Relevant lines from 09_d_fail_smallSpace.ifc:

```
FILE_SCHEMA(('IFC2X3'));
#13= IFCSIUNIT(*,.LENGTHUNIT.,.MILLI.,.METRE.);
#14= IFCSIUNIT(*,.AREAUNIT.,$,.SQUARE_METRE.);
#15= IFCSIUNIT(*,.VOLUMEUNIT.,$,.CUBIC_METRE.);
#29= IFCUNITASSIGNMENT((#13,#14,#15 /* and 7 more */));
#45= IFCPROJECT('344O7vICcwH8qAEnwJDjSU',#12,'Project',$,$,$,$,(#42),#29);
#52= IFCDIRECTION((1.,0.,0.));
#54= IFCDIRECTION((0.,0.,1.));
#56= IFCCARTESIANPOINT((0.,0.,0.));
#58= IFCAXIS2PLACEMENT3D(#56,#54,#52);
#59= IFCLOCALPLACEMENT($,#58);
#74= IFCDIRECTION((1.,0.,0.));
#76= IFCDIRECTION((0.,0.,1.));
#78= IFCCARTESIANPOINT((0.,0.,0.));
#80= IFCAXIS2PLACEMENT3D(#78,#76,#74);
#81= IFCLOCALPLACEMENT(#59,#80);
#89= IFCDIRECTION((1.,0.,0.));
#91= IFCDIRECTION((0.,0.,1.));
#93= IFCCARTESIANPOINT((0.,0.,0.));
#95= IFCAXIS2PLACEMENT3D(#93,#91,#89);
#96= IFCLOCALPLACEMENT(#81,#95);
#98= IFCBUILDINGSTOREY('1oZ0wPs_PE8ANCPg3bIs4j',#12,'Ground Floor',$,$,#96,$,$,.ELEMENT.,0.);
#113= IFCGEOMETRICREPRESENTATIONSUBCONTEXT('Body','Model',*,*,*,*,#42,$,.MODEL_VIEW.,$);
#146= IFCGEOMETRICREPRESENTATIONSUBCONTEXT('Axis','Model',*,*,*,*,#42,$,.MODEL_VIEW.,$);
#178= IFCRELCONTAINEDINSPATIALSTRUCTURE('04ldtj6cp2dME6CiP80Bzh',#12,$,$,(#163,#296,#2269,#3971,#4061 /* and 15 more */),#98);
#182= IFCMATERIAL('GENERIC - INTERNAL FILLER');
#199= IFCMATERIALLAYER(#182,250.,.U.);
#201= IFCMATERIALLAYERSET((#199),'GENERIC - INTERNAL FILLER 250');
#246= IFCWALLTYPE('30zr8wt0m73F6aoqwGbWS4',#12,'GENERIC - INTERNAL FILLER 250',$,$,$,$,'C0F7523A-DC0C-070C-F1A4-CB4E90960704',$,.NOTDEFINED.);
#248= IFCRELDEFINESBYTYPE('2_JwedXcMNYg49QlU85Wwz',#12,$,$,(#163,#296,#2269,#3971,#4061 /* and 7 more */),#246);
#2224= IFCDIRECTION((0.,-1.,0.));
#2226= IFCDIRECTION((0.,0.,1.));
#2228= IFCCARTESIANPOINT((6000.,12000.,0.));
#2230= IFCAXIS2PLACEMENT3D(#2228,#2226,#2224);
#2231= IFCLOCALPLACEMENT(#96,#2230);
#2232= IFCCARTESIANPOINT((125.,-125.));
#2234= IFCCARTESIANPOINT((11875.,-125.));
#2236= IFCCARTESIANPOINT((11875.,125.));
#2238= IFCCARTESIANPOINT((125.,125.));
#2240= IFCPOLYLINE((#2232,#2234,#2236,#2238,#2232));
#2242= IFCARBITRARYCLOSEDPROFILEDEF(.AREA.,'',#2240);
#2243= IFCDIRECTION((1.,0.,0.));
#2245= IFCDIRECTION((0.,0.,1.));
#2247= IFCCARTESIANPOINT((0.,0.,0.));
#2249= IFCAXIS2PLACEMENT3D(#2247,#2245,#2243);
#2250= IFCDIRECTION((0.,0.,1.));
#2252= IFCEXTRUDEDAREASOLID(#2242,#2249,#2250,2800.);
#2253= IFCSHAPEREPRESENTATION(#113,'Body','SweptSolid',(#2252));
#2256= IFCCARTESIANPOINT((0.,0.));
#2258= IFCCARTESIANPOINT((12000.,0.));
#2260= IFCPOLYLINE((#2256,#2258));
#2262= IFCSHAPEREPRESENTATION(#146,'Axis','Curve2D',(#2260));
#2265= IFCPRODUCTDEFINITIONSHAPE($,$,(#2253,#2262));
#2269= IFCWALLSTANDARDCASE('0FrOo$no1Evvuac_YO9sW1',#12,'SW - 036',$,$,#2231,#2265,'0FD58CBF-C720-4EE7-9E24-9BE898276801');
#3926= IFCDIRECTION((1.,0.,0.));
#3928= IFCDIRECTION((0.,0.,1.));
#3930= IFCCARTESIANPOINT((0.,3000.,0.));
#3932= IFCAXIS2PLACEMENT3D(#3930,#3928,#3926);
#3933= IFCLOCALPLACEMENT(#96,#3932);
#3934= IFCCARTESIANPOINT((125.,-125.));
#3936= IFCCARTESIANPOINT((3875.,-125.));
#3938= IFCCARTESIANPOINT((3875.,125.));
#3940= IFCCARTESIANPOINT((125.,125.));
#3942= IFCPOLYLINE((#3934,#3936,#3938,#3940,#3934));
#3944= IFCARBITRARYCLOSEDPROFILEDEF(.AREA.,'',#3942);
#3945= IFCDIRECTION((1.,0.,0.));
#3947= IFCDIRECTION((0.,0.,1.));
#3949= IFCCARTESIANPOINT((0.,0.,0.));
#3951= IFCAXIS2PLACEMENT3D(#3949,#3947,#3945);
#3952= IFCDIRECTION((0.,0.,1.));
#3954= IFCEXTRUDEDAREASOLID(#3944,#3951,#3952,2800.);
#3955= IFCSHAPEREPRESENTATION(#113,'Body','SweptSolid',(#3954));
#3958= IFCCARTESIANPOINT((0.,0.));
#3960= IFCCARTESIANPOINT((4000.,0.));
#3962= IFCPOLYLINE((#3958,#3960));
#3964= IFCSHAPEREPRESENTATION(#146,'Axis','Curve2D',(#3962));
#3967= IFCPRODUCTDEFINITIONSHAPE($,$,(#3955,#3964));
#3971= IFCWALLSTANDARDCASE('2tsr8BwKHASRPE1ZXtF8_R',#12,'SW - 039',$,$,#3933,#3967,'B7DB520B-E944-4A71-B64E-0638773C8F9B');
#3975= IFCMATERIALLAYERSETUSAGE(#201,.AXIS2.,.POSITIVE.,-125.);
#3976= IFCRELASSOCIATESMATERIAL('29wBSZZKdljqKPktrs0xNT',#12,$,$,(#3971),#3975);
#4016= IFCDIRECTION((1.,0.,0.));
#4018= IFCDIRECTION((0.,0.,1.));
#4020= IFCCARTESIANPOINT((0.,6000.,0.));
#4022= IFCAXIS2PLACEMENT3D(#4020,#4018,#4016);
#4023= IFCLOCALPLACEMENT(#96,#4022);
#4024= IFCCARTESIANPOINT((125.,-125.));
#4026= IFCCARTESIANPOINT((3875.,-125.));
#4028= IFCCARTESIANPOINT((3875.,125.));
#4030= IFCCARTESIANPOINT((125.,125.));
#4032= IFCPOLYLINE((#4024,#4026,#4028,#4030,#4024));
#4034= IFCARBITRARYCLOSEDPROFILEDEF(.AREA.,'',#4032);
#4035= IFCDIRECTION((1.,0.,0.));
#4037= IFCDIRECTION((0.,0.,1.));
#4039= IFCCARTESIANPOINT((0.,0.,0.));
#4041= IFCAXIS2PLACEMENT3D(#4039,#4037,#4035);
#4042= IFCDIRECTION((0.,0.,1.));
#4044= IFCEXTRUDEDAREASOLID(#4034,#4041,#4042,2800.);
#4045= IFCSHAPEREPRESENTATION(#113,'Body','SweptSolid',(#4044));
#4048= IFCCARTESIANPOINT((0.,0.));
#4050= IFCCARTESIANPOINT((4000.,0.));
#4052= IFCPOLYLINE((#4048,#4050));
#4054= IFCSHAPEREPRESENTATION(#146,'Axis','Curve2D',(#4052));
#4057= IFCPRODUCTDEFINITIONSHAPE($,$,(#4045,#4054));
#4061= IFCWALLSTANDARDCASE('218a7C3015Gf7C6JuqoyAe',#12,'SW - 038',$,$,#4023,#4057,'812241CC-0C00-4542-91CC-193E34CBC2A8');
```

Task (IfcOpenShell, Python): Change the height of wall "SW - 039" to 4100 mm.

```python
import ifcopenshell
import ifcopenshell.geom
import ifcopenshell.util.representation
import ifcopenshell.util.shape
import ifcopenshell.util.unit

model = ifcopenshell.open("09_d_fail_smallSpace.ifc")
unit_scale = ifcopenshell.util.unit.calculate_unit_scale(model)
settings = ifcopenshell.geom.settings()


def volume(element):
    """Net volume in cubic metres, openings subtracted."""
    shape = ifcopenshell.geom.create_shape(settings, element)
    return ifcopenshell.util.shape.get_volume(shape.geometry)


wall = model.by_id(3971)
before = volume(wall)

body = ifcopenshell.util.representation.get_representation(wall, "Model", "Body")
solid = body.Items[0]
old_height = solid.Depth
solid.Depth = 4.1 / unit_scale
after = volume(wall)

print(f"height {old_height:g} -> {solid.Depth:g}, volume {before:.3f} -> {after:.3f} m3")

model.write("09_d_fail_smallSpace_rev.ifc")
```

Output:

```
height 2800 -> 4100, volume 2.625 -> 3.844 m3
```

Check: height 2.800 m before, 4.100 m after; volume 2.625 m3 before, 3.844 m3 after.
